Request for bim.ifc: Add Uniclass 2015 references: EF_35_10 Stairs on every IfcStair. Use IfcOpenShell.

First a look at what the model holds.

```python
import ifcopenshell

model = ifcopenshell.open("bim.ifc")
print(model.schema)
print("classifications:", [c.Name for c in model.by_type("IfcClassification")])
for ifc_class in ("IfcDoor", "IfcRoof", "IfcStair", "IfcWall", "IfcWindow"):
    print(ifc_class, len(model.by_type(ifc_class)))
```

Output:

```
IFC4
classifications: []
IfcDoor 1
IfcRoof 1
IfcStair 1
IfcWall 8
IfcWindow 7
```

```python
import ifcopenshell
import ifcopenshell.api.classification

model = ifcopenshell.open("bim.ifc")

system = ifcopenshell.api.classification.add_classification(model, classification="Uniclass 2015")

codes = {
    "IfcStair": ("EF_35_10", "Stairs"),
}
for ifc_class, (code, name) in codes.items():
    products = model.by_type(ifc_class)
    ifcopenshell.api.classification.add_reference(
        model, products=products, classification=system, identification=code, name=name
    )
    print(code, len(products))

model.write("bim_v2.ifc")
```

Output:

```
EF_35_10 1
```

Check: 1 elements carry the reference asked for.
